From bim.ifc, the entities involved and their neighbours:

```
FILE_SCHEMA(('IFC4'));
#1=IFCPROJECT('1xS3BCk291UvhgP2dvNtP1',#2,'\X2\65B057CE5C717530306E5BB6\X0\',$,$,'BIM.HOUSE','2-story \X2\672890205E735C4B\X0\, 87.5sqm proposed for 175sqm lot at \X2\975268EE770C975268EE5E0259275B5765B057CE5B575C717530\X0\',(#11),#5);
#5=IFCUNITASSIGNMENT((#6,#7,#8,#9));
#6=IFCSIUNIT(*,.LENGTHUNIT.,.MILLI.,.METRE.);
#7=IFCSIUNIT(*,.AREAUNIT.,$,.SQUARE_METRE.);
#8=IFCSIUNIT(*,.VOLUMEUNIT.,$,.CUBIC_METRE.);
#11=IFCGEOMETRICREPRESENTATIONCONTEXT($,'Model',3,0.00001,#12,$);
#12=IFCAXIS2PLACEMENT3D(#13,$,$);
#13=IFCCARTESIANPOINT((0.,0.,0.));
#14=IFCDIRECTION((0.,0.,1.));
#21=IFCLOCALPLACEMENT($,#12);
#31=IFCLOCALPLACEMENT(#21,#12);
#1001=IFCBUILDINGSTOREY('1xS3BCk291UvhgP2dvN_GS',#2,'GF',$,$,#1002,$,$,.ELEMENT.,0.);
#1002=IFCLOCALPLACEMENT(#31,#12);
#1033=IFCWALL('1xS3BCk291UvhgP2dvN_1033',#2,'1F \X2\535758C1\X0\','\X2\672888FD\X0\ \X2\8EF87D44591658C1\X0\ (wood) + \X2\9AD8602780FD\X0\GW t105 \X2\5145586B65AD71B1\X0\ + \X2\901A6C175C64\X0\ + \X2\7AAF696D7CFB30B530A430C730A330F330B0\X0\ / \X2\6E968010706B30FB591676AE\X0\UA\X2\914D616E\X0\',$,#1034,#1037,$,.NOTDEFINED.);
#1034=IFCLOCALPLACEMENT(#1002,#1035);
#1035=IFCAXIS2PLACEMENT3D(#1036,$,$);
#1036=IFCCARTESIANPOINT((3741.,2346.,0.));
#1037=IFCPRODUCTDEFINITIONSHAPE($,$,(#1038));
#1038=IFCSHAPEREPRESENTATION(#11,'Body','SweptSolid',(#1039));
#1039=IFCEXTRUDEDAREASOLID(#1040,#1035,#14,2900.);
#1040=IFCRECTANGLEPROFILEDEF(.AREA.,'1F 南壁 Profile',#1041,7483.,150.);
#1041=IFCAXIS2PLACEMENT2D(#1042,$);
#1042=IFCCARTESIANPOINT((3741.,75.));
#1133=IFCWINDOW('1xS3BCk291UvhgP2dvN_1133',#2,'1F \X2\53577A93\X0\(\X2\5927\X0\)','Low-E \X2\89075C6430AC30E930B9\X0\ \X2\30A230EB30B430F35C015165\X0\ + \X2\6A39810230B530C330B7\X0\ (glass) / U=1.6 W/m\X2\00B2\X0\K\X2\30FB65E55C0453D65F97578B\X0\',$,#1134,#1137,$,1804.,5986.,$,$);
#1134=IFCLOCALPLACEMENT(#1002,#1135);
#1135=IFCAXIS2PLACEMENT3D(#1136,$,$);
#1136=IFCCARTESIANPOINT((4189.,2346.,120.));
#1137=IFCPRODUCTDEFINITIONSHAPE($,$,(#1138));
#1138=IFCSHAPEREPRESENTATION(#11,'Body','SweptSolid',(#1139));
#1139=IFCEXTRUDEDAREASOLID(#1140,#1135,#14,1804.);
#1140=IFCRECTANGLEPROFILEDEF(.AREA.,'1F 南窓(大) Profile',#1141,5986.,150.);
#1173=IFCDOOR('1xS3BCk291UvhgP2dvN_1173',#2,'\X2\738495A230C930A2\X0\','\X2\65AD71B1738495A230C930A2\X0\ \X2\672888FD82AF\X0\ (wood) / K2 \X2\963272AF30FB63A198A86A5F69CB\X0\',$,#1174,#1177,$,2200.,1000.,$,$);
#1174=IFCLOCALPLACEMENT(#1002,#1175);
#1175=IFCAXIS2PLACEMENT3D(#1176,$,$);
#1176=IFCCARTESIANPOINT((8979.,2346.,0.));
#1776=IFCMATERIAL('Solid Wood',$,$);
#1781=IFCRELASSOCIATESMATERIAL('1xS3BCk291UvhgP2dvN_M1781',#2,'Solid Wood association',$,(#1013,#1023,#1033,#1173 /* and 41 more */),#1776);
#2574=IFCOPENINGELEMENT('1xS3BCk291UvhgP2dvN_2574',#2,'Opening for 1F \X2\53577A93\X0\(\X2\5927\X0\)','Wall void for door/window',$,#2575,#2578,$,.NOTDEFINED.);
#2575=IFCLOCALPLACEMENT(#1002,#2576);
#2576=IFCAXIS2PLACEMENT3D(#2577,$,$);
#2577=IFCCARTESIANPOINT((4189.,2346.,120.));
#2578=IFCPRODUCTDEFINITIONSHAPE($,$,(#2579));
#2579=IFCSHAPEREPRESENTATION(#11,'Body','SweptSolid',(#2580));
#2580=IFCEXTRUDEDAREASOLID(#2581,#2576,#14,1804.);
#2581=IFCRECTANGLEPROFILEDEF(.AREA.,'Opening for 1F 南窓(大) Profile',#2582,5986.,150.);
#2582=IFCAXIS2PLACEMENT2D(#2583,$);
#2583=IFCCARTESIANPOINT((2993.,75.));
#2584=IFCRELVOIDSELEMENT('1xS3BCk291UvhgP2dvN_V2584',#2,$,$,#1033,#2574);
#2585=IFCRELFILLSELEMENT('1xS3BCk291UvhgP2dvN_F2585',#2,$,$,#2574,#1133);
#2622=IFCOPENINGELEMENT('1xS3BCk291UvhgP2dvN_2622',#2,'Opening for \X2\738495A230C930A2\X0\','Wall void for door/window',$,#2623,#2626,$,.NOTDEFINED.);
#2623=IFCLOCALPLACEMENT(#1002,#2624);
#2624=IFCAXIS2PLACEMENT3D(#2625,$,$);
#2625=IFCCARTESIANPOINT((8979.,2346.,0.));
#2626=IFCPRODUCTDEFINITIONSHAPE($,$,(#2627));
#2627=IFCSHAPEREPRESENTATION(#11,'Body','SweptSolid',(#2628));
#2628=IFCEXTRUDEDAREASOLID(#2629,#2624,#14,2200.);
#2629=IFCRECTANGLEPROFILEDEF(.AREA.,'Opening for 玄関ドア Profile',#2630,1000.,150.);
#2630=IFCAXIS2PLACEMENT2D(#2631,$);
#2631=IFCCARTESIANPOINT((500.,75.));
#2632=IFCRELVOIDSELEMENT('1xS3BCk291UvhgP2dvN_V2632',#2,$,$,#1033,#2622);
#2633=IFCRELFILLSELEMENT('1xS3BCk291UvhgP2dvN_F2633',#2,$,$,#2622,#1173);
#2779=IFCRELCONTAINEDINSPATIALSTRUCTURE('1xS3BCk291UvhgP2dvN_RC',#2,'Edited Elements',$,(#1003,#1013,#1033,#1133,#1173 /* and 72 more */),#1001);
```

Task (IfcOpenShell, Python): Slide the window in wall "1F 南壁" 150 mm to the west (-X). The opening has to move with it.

```python
import ifcopenshell
import ifcopenshell.api.geometry
import ifcopenshell.util.placement
import ifcopenshell.util.unit

model = ifcopenshell.open("bim.ifc")
unit_scale = ifcopenshell.util.unit.calculate_unit_scale(model)

window = model.by_id(1133)
opening = window.FillsVoids[0].RelatingOpeningElement
wall = opening.VoidsElements[0].RelatingBuildingElement

wall_matrix = ifcopenshell.util.placement.get_local_placement(wall.ObjectPlacement)
shift = wall_matrix[:3, 0] * -0.15 / unit_scale
before = ifcopenshell.util.placement.get_local_placement(window.ObjectPlacement)[:3, 3].copy()

# The window is not placed relative to its opening, so move both.
for product in (opening, window):
    matrix = ifcopenshell.util.placement.get_local_placement(product.ObjectPlacement)
    matrix[:3, 3] += shift
    ifcopenshell.api.geometry.edit_object_placement(model, product=product, matrix=matrix, is_si=False)

after = ifcopenshell.util.placement.get_local_placement(window.ObjectPlacement)[:3, 3]
print("window moved by", (after - before).round(3) + 0.0)

model.write("bim_updated.ifc")
```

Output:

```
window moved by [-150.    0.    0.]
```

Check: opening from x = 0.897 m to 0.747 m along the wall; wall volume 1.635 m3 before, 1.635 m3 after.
